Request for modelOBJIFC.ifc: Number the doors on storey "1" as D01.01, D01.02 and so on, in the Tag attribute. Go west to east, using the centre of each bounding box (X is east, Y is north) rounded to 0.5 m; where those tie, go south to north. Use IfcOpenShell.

First a look at what the model holds.

```python
import ifcopenshell
import ifcopenshell.util.element
import ifcopenshell.util.placement

model = ifcopenshell.open("modelOBJIFC.ifc")
print(model.schema)
storey = next(s for s in model.by_type("IfcBuildingStorey") if s.Name == "1")
doors = [e for e in ifcopenshell.util.element.get_decomposition(storey) if e.is_a("IfcDoor")]
for e in sorted(doors, key=lambda e: e.id()):
    origin = ifcopenshell.util.placement.get_local_placement(e.ObjectPlacement)[:3, 3]
    print(e.id(), e.Tag, e.Name, origin.round(2) + 0.0, sep=" | ")
```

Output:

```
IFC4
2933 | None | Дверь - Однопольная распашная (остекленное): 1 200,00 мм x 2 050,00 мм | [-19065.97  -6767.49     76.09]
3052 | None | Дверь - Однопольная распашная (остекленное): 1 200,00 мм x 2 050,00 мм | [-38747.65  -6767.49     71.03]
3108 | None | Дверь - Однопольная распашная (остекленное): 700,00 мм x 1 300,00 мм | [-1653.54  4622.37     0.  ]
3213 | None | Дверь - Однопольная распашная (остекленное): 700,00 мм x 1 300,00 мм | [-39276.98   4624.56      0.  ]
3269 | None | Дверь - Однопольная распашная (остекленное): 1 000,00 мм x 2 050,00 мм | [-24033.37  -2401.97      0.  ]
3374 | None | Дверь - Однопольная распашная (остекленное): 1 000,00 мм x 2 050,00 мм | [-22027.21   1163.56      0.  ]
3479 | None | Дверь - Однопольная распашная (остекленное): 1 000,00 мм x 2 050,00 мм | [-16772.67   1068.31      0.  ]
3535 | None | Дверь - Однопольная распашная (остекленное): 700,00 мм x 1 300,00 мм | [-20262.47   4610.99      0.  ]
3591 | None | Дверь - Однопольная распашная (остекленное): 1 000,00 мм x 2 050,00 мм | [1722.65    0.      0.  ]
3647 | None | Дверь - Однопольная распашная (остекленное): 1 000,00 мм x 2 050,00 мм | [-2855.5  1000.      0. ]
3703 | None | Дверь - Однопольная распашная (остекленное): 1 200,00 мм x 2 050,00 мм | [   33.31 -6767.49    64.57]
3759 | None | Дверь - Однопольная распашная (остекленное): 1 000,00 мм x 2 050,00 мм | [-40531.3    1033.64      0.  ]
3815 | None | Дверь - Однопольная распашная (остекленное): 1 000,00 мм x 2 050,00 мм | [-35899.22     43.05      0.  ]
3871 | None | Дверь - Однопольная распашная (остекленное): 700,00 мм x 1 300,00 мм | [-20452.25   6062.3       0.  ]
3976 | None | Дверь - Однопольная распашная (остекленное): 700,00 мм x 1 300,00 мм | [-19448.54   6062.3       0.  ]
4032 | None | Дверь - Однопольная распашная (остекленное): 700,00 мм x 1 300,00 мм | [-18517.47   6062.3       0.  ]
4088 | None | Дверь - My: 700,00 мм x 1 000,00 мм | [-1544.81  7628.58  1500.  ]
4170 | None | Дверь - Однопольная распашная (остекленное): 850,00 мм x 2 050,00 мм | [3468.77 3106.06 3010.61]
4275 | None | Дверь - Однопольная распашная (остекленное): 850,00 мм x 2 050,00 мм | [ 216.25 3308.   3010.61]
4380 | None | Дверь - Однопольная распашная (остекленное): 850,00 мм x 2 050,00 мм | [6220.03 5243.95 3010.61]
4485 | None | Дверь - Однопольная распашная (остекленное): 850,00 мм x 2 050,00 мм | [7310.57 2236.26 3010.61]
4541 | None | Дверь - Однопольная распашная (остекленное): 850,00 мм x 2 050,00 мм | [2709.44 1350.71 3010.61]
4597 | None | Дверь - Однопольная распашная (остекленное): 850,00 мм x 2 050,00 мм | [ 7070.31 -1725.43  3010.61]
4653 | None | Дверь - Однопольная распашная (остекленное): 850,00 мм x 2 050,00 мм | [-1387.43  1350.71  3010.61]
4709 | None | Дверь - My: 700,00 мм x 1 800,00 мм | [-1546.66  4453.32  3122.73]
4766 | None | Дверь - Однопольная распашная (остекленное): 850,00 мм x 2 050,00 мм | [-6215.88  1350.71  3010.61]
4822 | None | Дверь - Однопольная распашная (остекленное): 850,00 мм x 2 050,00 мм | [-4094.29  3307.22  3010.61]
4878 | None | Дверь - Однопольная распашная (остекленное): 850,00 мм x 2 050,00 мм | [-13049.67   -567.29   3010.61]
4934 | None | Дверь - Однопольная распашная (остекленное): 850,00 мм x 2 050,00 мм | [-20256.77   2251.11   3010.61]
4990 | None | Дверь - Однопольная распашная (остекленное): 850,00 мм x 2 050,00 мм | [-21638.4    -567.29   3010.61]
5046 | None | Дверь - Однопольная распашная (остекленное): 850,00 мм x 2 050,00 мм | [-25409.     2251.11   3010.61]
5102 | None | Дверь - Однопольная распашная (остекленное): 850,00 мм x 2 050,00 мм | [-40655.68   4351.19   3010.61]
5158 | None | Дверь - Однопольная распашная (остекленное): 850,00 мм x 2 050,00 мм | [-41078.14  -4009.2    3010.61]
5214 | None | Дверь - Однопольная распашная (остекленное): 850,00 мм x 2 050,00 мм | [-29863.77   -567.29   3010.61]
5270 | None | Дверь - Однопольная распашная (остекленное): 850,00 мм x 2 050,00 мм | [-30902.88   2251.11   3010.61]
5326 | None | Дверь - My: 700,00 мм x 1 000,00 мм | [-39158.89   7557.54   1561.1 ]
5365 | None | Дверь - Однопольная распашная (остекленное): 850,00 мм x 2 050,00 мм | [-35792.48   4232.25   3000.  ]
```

```python
import ifcopenshell
import ifcopenshell.geom
import ifcopenshell.util.element
import ifcopenshell.util.shape

model = ifcopenshell.open("modelOBJIFC.ifc")
settings = ifcopenshell.geom.settings()
settings.set("use-world-coords", True)


def centre(element):
    shape = ifcopenshell.geom.create_shape(settings, element)
    return ifcopenshell.util.shape.get_bbox_centroid(shape.geometry)


storey = next(s for s in model.by_type("IfcBuildingStorey") if s.Name == "1")
doors = [e for e in ifcopenshell.util.element.get_decomposition(storey) if e.is_a("IfcDoor")]

# Insertion points can sit at a corner or the storey origin, so sort by the geometry (in metres).
centres = {e: centre(e) for e in doors}
doors.sort(key=lambda e: (round(centres[e][0] / 0.5), centres[e][1]))

for i, e in enumerate(doors, start=1):
    number = f"D01.{i:02d}"
    e.Tag = number
    print(e.id(), number)

model.write("modelOBJIFC-out.ifc")
```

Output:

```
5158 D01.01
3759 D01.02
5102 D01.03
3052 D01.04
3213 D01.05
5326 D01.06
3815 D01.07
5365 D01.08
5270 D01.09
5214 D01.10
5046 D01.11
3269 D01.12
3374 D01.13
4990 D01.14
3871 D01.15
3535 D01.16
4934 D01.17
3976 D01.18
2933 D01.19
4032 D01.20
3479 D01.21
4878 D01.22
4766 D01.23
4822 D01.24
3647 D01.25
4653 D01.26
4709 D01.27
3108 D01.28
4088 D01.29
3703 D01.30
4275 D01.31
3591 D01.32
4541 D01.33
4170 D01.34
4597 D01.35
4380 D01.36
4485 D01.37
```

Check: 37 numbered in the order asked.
